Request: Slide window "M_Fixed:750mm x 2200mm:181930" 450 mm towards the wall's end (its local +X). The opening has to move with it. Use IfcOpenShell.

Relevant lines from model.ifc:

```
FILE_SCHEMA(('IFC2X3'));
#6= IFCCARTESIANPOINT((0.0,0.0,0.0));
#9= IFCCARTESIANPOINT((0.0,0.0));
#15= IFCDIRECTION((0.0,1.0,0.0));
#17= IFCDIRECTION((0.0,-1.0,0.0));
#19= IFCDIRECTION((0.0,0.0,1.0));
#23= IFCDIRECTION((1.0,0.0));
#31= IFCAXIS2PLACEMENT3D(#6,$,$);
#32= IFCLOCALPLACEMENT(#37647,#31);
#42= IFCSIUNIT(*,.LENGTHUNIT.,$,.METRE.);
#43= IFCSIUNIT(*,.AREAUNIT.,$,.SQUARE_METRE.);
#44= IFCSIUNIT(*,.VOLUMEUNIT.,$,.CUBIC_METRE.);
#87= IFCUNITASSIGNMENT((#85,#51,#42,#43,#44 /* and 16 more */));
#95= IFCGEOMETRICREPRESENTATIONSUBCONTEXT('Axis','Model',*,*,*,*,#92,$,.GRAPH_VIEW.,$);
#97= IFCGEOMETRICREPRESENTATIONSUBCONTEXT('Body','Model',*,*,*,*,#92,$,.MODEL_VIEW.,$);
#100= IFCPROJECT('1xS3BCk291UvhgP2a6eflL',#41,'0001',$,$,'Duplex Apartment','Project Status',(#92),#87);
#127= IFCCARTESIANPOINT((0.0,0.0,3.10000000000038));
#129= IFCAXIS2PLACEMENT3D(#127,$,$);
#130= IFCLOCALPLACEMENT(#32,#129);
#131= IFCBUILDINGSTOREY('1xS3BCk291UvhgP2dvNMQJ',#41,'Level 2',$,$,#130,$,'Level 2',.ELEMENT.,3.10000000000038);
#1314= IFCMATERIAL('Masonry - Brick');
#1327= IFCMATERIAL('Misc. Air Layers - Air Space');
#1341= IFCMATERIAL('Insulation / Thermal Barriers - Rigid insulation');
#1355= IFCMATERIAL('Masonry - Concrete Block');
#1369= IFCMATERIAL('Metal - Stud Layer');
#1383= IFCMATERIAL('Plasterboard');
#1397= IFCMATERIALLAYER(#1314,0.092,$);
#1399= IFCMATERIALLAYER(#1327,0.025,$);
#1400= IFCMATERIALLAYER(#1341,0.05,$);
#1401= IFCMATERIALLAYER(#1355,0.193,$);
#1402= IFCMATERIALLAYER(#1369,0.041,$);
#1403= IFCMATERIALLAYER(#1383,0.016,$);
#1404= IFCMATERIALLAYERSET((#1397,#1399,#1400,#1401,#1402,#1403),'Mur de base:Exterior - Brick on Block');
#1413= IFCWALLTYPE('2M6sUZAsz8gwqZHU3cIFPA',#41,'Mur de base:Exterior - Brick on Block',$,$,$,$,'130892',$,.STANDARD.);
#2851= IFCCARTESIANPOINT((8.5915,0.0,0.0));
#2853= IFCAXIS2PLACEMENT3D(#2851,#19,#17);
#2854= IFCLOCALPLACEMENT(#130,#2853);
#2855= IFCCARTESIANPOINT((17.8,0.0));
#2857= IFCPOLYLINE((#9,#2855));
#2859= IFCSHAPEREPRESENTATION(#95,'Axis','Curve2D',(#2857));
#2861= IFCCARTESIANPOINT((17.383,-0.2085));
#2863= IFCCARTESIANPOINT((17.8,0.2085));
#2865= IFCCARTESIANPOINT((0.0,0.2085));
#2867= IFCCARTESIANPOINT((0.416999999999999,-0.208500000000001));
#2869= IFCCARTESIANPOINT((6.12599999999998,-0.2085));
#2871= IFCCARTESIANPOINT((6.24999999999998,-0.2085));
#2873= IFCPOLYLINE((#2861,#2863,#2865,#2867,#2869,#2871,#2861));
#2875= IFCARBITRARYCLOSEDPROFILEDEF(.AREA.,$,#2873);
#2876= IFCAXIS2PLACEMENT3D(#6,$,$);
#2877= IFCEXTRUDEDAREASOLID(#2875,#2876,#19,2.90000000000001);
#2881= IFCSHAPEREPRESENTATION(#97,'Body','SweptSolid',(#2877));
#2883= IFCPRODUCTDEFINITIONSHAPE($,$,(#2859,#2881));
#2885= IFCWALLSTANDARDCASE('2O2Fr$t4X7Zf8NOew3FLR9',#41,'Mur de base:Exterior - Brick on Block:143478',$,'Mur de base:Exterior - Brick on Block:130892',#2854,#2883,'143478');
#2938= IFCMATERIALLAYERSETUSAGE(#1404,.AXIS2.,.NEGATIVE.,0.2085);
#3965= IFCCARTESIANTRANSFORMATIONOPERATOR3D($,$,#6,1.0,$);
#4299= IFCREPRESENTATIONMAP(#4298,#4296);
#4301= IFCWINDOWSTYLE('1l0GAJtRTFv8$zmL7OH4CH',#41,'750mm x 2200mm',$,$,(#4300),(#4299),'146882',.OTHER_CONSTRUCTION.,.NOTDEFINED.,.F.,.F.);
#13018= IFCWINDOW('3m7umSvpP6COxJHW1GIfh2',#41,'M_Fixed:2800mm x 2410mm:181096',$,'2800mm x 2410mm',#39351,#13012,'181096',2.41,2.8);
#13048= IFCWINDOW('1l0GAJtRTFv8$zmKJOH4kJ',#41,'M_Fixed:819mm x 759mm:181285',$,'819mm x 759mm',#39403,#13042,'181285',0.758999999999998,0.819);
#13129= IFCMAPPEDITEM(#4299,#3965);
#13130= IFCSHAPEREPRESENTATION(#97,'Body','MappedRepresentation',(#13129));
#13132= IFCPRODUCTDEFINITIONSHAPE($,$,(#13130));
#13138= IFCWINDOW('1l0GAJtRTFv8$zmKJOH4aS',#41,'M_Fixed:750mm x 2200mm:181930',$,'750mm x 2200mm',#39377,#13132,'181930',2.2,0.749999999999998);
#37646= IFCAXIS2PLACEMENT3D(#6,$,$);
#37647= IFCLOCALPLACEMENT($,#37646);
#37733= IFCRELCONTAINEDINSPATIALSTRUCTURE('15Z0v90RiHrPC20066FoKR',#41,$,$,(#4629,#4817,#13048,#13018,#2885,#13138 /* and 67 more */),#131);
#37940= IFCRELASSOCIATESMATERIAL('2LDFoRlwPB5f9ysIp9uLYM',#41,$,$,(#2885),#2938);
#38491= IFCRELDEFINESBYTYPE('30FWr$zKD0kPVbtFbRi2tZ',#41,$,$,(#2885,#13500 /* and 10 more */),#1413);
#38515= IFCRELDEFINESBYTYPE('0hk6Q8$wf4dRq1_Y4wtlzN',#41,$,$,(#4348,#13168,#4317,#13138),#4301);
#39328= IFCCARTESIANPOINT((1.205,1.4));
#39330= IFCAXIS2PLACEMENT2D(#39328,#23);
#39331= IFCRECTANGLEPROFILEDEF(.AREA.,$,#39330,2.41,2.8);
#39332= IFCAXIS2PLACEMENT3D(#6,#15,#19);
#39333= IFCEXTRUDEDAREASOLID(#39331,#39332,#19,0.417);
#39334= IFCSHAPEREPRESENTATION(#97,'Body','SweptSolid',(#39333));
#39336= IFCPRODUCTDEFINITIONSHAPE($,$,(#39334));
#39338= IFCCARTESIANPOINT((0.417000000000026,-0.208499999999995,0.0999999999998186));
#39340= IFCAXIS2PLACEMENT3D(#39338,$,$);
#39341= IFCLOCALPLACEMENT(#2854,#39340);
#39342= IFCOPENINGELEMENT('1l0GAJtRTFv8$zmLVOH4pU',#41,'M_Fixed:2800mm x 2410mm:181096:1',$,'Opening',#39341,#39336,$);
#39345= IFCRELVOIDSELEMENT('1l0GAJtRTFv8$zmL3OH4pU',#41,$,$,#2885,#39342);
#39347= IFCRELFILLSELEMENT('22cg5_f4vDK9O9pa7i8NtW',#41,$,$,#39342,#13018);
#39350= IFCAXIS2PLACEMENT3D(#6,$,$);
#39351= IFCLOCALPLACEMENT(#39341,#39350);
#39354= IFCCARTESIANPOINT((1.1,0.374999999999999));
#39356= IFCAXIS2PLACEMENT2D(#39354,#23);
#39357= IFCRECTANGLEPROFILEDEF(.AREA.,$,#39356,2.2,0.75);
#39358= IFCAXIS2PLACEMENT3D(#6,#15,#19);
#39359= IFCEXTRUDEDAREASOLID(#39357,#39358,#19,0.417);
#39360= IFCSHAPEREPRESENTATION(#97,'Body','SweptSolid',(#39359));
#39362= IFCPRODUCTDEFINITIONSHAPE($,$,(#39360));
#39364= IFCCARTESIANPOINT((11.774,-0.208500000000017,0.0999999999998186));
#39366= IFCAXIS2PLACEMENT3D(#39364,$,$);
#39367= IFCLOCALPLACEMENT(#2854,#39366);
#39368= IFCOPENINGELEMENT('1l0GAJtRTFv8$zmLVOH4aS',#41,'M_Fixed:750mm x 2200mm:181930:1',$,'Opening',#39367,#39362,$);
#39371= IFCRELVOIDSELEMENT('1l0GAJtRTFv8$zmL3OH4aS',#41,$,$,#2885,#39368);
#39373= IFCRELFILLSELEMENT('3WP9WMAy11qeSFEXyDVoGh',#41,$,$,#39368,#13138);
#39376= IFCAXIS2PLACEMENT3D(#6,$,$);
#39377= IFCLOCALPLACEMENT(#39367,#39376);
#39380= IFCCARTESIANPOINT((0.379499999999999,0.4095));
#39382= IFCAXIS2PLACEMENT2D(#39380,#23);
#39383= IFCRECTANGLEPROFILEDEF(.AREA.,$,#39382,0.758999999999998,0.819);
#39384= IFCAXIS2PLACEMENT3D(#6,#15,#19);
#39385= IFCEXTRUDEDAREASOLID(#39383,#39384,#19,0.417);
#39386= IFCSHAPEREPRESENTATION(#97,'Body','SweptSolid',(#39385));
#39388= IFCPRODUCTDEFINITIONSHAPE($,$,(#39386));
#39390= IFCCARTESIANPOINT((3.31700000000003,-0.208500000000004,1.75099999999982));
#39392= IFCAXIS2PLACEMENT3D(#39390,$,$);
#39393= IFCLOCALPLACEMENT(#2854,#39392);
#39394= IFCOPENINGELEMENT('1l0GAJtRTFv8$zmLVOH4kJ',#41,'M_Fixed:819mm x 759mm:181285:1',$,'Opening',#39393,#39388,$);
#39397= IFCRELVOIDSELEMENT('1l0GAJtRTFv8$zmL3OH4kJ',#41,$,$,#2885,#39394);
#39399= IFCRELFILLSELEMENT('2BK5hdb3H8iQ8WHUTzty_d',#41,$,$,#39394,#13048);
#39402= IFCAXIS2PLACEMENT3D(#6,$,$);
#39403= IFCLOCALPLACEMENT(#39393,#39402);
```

```python
import ifcopenshell
import ifcopenshell.api.geometry
import ifcopenshell.util.placement

model = ifcopenshell.open("model.ifc")

window = model.by_guid("1l0GAJtRTFv8$zmKJOH4aS")
opening = window.FillsVoids[0].RelatingOpeningElement
wall = opening.VoidsElements[0].RelatingBuildingElement

wall_matrix = ifcopenshell.util.placement.get_local_placement(wall.ObjectPlacement)
shift = wall_matrix[:3, 0] * 0.45
before = ifcopenshell.util.placement.get_local_placement(window.ObjectPlacement)[:3, 3].copy()

# The window is placed relative to its opening, so it follows when the opening moves.
matrix = ifcopenshell.util.placement.get_local_placement(opening.ObjectPlacement)
matrix[:3, 3] += shift
ifcopenshell.api.geometry.edit_object_placement(
    model, product=opening, matrix=matrix, is_si=False, should_transform_children=True
)

after = ifcopenshell.util.placement.get_local_placement(window.ObjectPlacement)[:3, 3]
print("window moved by", (after - before).round(3) + 0.0)

model.write("model_edited.ifc")
```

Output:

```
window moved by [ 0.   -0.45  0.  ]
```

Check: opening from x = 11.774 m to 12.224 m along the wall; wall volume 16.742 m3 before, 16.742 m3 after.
